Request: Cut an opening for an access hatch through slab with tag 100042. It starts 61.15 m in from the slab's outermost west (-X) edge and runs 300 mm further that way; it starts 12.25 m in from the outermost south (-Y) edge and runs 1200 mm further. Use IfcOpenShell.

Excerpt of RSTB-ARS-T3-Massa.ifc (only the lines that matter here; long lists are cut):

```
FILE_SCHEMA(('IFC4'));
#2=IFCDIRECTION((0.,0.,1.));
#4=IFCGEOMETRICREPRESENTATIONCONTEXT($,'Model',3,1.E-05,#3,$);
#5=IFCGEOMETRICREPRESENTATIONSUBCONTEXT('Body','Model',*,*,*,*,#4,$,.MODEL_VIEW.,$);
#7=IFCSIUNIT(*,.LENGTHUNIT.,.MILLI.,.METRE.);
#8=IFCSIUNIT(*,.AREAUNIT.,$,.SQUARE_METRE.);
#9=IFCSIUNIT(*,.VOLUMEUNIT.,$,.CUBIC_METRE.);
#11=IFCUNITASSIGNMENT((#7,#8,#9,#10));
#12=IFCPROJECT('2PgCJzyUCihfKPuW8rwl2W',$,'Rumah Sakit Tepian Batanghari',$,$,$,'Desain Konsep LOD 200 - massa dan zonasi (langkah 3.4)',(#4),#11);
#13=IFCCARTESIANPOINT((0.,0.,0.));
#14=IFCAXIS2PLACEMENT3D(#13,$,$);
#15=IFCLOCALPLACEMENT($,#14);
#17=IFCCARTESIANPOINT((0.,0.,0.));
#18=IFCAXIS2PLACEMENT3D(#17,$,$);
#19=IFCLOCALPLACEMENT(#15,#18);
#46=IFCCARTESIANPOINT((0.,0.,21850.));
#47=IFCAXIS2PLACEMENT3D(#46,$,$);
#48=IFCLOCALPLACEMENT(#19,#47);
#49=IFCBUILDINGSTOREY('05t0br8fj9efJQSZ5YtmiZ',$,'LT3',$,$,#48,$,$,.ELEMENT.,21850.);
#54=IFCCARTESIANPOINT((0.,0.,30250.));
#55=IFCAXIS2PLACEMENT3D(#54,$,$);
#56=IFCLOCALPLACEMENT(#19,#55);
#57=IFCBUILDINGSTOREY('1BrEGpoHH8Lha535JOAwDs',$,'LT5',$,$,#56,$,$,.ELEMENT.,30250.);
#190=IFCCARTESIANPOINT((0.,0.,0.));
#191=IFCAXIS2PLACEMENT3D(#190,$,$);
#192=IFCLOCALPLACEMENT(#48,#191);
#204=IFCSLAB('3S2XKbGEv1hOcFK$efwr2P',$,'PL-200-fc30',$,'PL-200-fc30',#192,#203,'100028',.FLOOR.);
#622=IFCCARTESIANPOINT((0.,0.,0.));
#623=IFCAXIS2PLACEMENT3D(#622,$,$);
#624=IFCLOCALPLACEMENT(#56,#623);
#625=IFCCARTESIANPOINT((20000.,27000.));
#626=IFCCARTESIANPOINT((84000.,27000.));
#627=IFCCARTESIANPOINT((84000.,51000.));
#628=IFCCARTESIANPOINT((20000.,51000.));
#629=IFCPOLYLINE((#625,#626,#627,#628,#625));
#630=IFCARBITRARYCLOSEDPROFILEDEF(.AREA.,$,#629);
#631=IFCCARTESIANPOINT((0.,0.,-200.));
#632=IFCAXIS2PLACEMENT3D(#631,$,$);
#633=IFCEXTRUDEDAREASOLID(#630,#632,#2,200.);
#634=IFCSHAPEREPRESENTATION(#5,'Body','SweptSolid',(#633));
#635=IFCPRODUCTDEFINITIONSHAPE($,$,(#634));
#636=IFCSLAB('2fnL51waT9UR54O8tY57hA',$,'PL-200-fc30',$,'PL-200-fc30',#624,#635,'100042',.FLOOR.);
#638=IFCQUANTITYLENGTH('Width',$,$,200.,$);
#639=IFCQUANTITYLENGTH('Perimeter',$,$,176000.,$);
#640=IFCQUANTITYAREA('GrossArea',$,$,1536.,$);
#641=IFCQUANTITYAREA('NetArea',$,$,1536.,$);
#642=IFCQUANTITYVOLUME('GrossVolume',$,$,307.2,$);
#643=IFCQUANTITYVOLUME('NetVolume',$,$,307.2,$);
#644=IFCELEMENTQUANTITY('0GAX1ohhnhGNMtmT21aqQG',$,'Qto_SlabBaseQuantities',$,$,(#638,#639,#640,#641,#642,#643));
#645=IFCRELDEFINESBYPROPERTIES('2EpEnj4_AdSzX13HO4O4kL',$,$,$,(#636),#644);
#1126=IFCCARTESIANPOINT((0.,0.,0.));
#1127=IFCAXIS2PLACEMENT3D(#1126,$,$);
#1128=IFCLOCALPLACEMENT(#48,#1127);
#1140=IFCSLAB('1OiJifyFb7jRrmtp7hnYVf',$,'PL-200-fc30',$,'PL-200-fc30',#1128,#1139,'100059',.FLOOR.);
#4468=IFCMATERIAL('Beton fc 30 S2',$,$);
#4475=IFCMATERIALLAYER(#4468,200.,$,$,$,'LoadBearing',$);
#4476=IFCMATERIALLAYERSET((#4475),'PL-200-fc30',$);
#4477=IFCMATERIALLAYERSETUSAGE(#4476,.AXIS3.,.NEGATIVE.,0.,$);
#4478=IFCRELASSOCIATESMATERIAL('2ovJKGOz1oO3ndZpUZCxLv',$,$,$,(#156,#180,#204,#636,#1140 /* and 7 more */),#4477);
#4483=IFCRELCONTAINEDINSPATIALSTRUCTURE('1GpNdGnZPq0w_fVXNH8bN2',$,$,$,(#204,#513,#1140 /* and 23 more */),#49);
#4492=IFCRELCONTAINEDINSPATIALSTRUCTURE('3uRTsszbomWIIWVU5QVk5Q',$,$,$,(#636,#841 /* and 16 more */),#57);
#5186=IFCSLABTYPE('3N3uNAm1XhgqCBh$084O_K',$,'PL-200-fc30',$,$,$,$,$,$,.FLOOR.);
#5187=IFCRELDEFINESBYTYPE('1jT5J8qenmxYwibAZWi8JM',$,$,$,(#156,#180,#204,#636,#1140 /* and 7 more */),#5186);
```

```python
import numpy as np
import ifcopenshell
import ifcopenshell.api.feature
import ifcopenshell.api.geometry
import ifcopenshell.api.pset
import ifcopenshell.api.root
import ifcopenshell.geom
import ifcopenshell.util.element
import ifcopenshell.util.placement
import ifcopenshell.util.representation
import ifcopenshell.util.shape
import ifcopenshell.util.unit

model = ifcopenshell.open("RSTB-ARS-T3-Massa.ifc")
unit_scale = ifcopenshell.util.unit.calculate_unit_scale(model)
area_scale = ifcopenshell.util.unit.calculate_unit_scale(model, "AREAUNIT")
volume_scale = ifcopenshell.util.unit.calculate_unit_scale(model, "VOLUMEUNIT")
settings = ifcopenshell.geom.settings()


def volume(element):
    """Net volume in cubic metres, openings subtracted."""
    shape = ifcopenshell.geom.create_shape(settings, element)
    return ifcopenshell.util.shape.get_volume(shape.geometry)


slab = model.by_id(636)
before = volume(slab)

# Extent in the slab's own axes, in metres. The edges named are its -X and -Y sides.
slab_shape = ifcopenshell.geom.create_shape(settings, slab)
vertices = ifcopenshell.util.shape.get_vertices(slab_shape.geometry)
x_min, y_min, bottom = vertices.min(axis=0)
top = vertices[:, 2].max()

opening = ifcopenshell.api.root.create_entity(model, ifc_class="IfcOpeningElement", name="Access hatch opening", predefined_type="OPENING")
context = ifcopenshell.util.representation.get_context(model, "Model", "Body", "MODEL_VIEW")
width, depth = 0.3, 1.2
outline = [(0.0, 0.0), (width, 0.0), (width, depth), (0.0, depth), (0.0, 0.0)]
# Overshoot both faces by 50 mm so the cut is clean.
shape = ifcopenshell.api.geometry.add_slab_representation(
    model, context=context, depth=top - bottom + 0.1, polyline=outline
)
ifcopenshell.api.geometry.assign_representation(model, product=opening, representation=shape)

matrix = ifcopenshell.util.placement.get_local_placement(slab.ObjectPlacement)
matrix[:, 3] = matrix @ np.append(np.array([x_min + 61.15, y_min + 12.25, bottom - 0.05]) / unit_scale, 1.0)
ifcopenshell.api.geometry.edit_object_placement(model, product=opening, matrix=matrix, is_si=False)
ifcopenshell.api.feature.add_feature(model, feature=opening, element=slab)

after = volume(slab)

# Update the slab's stored quantities.
qto = model.by_id(ifcopenshell.util.element.get_pset(slab, "Qto_SlabBaseQuantities", should_inherit=False)["id"])
ifcopenshell.api.pset.edit_qto(model, qto=qto, properties={
    "NetArea": after / (top - bottom) / area_scale,
    "NetVolume": after / volume_scale,
})

print(f"slab volume {before:.3f} -> {after:.3f} m3")

model.write("RSTB-ARS-T3-Massa_edited.ifc")
```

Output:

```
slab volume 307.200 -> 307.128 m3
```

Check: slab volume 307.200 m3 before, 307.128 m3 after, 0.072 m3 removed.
